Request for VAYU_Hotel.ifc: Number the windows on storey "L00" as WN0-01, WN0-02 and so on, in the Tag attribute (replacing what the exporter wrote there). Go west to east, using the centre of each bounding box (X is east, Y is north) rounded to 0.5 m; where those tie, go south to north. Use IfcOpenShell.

First a look at what the model holds.

```python
import ifcopenshell
import ifcopenshell.util.element
import ifcopenshell.util.placement

model = ifcopenshell.open("VAYU_Hotel.ifc")
print(model.schema)
storey = next(s for s in model.by_type("IfcBuildingStorey") if s.Name == "L00")
windows = [e for e in ifcopenshell.util.element.get_decomposition(storey) if e.is_a("IfcWindow")]
for e in sorted(windows, key=lambda e: e.id()):
    origin = ifcopenshell.util.placement.get_local_placement(e.ObjectPlacement)[:3, 3]
    print(e.id(), e.Tag, e.Name, origin.round(2) + 0.0, sep=" | ")
```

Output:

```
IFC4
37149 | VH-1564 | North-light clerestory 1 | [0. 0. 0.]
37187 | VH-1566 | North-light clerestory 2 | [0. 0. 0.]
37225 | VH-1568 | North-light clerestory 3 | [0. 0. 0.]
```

```python
import ifcopenshell
import ifcopenshell.geom
import ifcopenshell.util.element
import ifcopenshell.util.shape

model = ifcopenshell.open("VAYU_Hotel.ifc")
settings = ifcopenshell.geom.settings()
settings.set("use-world-coords", True)


def centre(element):
    shape = ifcopenshell.geom.create_shape(settings, element)
    return ifcopenshell.util.shape.get_bbox_centroid(shape.geometry)


storey = next(s for s in model.by_type("IfcBuildingStorey") if s.Name == "L00")
windows = [e for e in ifcopenshell.util.element.get_decomposition(storey) if e.is_a("IfcWindow")]

# Insertion points can sit at a corner or the storey origin, so sort by the geometry (in metres).
centres = {e: centre(e) for e in windows}
windows.sort(key=lambda e: (round(centres[e][0] / 0.5), centres[e][1]))

for i, e in enumerate(windows, start=1):
    number = f"WN0-{i:02d}"
    e.Tag = number
    print(e.id(), number)

model.write("VAYU_Hotel_rev.ifc")
```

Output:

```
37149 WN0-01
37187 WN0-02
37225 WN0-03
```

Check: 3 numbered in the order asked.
